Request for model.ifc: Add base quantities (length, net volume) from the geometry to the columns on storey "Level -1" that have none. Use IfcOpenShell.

First a look at what the model holds.

```python
import ifcopenshell
import ifcopenshell.util.element
import ifcopenshell.util.unit

model = ifcopenshell.open("model.ifc")
print(model.schema)
for unit_type in ("LENGTHUNIT", "AREAUNIT", "VOLUMEUNIT"):
    print(unit_type, ifcopenshell.util.unit.calculate_unit_scale(model, unit_type))
storey = next(s for s in model.by_type("IfcBuildingStorey") if s.Name == "Level -1")
columns = [e for e in ifcopenshell.util.element.get_decomposition(storey) if e.is_a("IfcColumn")]
for e in sorted(columns, key=lambda e: e.id()):
    print(e.id(), e.is_a(), e.Name, list(ifcopenshell.util.element.get_psets(e, qtos_only=True)), sep=" | ")
```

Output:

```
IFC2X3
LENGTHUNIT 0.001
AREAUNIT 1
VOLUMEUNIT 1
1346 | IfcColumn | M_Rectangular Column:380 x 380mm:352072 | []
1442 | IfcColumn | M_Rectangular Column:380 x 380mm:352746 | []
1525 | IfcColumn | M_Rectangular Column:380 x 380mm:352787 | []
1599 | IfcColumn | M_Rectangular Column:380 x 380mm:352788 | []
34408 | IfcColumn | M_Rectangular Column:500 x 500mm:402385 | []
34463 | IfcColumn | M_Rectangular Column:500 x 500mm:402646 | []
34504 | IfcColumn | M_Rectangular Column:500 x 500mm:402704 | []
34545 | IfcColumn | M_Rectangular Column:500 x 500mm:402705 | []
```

```python
import ifcopenshell
import ifcopenshell.api.pset
import ifcopenshell.geom
import ifcopenshell.util.element
import ifcopenshell.util.shape
import ifcopenshell.util.unit

model = ifcopenshell.open("model.ifc")
unit_scale = ifcopenshell.util.unit.calculate_unit_scale(model)
volume_scale = ifcopenshell.util.unit.calculate_unit_scale(model, "VOLUMEUNIT")
settings = ifcopenshell.geom.settings()

storey = next(s for s in model.by_type("IfcBuildingStorey") if s.Name == "Level -1")
columns = [e for e in ifcopenshell.util.element.get_decomposition(storey) if e.is_a("IfcColumn")]

for e in sorted(columns, key=lambda e: e.id()):
    if ifcopenshell.util.element.get_psets(e, qtos_only=True, should_inherit=False):
        continue
    # Geometry comes back in metres, in the element's own axes.
    shape = ifcopenshell.geom.create_shape(settings, e)
    values = {
        "Length": ifcopenshell.util.shape.get_z(shape.geometry) / unit_scale,
        "NetVolume": ifcopenshell.util.shape.get_volume(shape.geometry) / volume_scale,
    }
    qto = ifcopenshell.api.pset.add_qto(model, product=e, name="BaseQuantities")
    ifcopenshell.api.pset.edit_qto(model, qto=qto, properties=values)
    print(e.id(), {k: round(v, 3) for k, v in values.items()})

model.write("model-out.ifc")
```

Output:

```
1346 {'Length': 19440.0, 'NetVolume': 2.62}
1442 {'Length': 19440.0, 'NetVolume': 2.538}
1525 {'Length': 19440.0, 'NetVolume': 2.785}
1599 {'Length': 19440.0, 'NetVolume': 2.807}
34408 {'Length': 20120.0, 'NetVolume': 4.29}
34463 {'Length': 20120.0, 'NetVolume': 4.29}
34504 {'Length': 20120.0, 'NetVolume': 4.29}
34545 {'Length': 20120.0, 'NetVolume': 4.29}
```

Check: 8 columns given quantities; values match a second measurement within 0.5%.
